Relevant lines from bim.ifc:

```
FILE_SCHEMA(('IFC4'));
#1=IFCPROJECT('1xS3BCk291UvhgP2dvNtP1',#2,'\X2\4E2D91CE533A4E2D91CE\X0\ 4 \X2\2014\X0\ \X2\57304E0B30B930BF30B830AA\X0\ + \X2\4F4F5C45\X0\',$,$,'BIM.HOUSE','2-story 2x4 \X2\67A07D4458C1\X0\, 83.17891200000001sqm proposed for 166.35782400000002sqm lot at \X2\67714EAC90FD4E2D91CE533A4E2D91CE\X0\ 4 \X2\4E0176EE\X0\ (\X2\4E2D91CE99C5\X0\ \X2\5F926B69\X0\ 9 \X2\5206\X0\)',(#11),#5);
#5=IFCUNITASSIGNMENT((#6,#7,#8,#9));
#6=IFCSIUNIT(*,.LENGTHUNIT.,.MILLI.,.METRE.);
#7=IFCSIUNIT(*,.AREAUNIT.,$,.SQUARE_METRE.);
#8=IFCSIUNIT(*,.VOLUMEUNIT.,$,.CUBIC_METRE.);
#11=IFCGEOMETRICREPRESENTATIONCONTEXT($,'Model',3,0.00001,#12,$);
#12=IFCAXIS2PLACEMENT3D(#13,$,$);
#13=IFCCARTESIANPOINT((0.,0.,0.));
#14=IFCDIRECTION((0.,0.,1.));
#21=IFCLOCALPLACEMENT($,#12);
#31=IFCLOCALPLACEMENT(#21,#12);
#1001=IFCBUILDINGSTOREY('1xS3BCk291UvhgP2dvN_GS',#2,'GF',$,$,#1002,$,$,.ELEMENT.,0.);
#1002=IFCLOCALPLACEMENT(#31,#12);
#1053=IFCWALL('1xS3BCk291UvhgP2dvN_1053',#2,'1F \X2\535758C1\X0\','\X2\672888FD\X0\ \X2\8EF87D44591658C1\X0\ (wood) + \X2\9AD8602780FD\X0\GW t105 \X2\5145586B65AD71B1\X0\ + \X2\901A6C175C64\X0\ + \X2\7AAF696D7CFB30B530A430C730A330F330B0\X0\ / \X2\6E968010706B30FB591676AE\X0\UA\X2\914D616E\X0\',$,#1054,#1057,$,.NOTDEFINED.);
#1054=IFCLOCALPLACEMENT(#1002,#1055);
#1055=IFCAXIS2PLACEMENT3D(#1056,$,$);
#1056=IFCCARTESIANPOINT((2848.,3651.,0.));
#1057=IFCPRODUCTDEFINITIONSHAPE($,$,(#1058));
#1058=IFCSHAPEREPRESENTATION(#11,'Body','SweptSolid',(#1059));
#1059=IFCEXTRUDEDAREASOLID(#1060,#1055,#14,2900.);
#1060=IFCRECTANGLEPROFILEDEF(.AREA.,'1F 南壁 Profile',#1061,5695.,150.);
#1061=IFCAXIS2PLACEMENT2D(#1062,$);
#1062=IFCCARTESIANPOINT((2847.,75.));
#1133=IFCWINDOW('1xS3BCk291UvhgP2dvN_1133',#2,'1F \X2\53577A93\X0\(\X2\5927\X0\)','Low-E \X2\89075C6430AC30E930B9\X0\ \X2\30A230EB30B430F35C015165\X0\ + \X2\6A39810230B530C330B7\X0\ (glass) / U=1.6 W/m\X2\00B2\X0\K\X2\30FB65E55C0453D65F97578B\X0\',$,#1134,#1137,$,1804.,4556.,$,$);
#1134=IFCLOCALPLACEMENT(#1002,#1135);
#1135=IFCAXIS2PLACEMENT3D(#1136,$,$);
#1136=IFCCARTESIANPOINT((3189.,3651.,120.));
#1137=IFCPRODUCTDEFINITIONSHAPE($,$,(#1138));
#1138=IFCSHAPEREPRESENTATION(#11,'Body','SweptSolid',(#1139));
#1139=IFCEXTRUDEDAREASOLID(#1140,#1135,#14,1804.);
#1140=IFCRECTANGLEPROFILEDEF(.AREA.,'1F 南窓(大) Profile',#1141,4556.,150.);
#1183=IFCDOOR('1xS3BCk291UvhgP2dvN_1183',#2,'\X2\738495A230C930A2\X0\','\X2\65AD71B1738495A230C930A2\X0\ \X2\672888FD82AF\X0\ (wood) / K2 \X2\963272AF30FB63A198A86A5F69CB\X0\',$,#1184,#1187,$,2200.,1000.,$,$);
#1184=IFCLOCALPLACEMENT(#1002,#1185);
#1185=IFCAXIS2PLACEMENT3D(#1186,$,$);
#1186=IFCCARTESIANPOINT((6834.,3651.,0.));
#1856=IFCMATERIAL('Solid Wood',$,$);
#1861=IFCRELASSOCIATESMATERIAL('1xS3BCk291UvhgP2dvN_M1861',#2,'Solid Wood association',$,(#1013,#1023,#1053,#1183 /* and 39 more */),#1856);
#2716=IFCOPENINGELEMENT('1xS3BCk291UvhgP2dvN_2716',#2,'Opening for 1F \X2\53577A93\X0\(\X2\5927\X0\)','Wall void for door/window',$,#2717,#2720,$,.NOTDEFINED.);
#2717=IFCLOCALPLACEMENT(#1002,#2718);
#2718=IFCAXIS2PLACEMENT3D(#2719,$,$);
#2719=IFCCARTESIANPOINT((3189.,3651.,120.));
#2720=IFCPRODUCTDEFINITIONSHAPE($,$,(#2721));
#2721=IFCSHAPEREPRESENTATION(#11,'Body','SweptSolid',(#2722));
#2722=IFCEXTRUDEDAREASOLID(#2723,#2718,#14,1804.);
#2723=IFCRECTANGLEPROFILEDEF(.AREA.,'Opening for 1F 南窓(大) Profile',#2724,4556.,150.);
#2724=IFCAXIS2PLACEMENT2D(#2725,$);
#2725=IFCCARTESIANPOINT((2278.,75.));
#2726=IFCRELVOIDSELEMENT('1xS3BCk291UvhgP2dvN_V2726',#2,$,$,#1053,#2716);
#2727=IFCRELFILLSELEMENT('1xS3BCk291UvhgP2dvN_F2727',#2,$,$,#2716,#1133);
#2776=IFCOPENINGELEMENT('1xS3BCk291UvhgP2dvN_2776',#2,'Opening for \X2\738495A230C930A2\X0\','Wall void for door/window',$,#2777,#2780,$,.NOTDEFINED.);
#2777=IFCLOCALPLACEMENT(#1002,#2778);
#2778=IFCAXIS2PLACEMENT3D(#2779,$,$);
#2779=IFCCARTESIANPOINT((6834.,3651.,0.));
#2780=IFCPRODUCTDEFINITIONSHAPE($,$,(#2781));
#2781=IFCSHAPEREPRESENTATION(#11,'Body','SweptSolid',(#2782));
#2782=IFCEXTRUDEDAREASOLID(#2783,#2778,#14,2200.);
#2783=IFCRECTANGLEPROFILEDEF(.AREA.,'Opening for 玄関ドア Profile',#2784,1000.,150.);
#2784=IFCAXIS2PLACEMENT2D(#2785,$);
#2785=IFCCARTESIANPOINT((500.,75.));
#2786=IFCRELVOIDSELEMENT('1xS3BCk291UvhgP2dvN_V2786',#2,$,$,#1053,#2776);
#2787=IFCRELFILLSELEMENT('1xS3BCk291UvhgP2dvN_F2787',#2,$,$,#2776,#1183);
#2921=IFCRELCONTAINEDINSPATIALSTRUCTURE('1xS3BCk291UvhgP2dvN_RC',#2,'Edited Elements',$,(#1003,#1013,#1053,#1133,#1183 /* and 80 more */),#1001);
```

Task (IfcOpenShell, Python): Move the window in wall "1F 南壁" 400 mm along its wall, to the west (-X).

```python
import ifcopenshell
import ifcopenshell.api.geometry
import ifcopenshell.util.placement
import ifcopenshell.util.unit

model = ifcopenshell.open("bim.ifc")
unit_scale = ifcopenshell.util.unit.calculate_unit_scale(model)

window = model.by_guid("1xS3BCk291UvhgP2dvN_1133")
opening = window.FillsVoids[0].RelatingOpeningElement
wall = opening.VoidsElements[0].RelatingBuildingElement

wall_matrix = ifcopenshell.util.placement.get_local_placement(wall.ObjectPlacement)
shift = wall_matrix[:3, 0] * -0.4 / unit_scale
before = ifcopenshell.util.placement.get_local_placement(window.ObjectPlacement)[:3, 3].copy()

# The window is not placed relative to its opening, so move both.
for product in (opening, window):
    matrix = ifcopenshell.util.placement.get_local_placement(product.ObjectPlacement)
    matrix[:3, 3] += shift
    ifcopenshell.api.geometry.edit_object_placement(model, product=product, matrix=matrix, is_si=False)

after = ifcopenshell.util.placement.get_local_placement(window.ObjectPlacement)[:3, 3]
print("window moved by", (after - before).round(3) + 0.0)

model.write("bim_rev.ifc")
```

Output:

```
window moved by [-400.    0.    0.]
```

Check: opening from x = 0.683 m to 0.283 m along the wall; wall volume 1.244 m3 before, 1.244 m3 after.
